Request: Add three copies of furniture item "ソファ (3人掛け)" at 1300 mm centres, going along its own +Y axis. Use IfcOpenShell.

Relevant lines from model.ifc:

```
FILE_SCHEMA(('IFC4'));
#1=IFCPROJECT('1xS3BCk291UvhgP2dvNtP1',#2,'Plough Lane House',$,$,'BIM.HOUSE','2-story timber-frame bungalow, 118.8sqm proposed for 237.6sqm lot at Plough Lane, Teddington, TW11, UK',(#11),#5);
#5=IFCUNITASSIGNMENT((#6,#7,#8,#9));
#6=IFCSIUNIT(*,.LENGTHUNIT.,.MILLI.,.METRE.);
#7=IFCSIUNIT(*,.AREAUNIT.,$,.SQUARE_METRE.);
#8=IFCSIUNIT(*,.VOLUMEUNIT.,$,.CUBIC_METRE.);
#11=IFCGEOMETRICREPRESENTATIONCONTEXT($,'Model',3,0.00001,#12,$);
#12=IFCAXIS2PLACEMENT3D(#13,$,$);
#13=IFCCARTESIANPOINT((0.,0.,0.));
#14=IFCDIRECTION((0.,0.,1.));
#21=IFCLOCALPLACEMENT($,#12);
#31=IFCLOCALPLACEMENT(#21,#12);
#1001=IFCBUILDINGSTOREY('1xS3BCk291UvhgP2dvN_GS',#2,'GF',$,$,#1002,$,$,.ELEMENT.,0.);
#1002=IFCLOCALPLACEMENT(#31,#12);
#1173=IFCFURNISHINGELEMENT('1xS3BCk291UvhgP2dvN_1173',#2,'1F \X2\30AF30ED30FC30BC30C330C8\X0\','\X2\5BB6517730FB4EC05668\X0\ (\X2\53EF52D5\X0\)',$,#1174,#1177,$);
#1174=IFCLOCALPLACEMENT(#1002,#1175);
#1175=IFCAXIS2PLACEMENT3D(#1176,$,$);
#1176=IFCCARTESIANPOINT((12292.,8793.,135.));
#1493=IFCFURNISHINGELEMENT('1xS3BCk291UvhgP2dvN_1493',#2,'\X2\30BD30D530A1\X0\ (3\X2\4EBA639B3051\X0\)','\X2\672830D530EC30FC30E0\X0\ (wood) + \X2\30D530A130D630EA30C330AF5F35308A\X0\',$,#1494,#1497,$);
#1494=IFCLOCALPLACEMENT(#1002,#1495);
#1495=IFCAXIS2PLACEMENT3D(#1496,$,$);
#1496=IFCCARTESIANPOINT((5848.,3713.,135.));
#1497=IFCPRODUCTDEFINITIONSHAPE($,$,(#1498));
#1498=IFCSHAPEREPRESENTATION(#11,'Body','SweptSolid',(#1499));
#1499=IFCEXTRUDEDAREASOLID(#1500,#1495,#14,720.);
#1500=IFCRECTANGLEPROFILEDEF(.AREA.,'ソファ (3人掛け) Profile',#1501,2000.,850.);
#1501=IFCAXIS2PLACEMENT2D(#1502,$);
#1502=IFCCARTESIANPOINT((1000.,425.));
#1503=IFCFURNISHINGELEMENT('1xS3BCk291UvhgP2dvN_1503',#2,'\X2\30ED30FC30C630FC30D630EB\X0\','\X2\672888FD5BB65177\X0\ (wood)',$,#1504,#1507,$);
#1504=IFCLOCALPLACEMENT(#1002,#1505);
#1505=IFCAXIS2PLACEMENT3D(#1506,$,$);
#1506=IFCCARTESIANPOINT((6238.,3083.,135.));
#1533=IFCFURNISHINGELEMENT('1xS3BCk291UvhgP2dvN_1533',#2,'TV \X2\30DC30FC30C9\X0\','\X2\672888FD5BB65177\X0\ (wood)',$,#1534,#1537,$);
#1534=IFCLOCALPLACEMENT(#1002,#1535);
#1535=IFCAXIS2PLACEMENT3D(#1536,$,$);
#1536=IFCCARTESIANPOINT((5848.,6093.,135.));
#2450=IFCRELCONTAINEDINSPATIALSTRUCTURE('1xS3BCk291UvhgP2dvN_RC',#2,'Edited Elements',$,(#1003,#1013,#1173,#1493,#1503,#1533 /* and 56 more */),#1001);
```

```python
import ifcopenshell
import ifcopenshell.api.geometry
import ifcopenshell.api.root
import ifcopenshell.util.element
import ifcopenshell.util.placement
import ifcopenshell.util.unit

model = ifcopenshell.open("model.ifc")
unit_scale = ifcopenshell.util.unit.calculate_unit_scale(model)


def reuse_history(source, copy):
    """copy_class also copies each property set's owner history, people and application; keep the originals."""
    for rel in copy.IsDefinedBy:
        if rel.is_a("IfcRelDefinesByProperties") and (history := rel.RelatingPropertyDefinition.OwnerHistory):
            rel.RelatingPropertyDefinition.OwnerHistory = source.OwnerHistory
            ifcopenshell.util.element.remove_deep2(model, history)


source = model.by_id(1493)
base = ifcopenshell.util.placement.get_local_placement(source.ObjectPlacement)
step = base[:3, 1] * 1.3 / unit_scale

for i in range(1, 4):
    copy = ifcopenshell.api.root.copy_class(model, product=source)
    copy.Representation = ifcopenshell.util.element.copy_deep(
        model, source.Representation, exclude=["IfcGeometricRepresentationContext", "IfcRepresentationMap"]
    )
    reuse_history(source, copy)
    matrix = base.copy()
    matrix[:3, 3] += i * step
    print("added at", matrix[:3, 3].round(3) + 0.0)
    ifcopenshell.api.geometry.edit_object_placement(model, product=copy, matrix=matrix, is_si=False)

model.write("model_v2.ifc")
```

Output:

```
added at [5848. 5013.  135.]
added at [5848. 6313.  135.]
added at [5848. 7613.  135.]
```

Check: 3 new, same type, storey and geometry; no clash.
